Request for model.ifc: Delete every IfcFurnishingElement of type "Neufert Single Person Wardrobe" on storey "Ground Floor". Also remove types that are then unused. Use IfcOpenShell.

First a look at what the model holds.

```python
import ifcopenshell
import ifcopenshell.util.element

model = ifcopenshell.open("model.ifc")
print(model.schema)
storey = next(s for s in model.by_type("IfcBuildingStorey") if s.Name == "Ground Floor")
furniture = [e for e in ifcopenshell.util.element.get_decomposition(storey) if e.is_a("IfcFurnishingElement")]
seen = {}
for e in furniture:
    element_type = ifcopenshell.util.element.get_type(e)
    name = element_type.Name if element_type not in (None, e) else None
    seen[name] = seen.get(name, 0) + 1
for name, count in sorted(seen.items(), key=str):
    print(count, "x", name)
```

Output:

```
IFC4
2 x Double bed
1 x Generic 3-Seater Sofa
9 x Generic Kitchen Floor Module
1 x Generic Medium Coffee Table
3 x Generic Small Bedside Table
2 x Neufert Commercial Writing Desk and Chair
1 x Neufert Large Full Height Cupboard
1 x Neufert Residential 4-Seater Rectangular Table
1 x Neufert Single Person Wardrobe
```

```python
import ifcopenshell
import ifcopenshell.api.root
import ifcopenshell.util.element

model = ifcopenshell.open("model.ifc")

storey = next(s for s in model.by_type("IfcBuildingStorey") if s.Name == "Ground Floor")
furniture = [e for e in ifcopenshell.util.element.get_decomposition(storey) if e.is_a("IfcFurnishingElement")]
targets = [e for e in furniture if (t := ifcopenshell.util.element.get_type(e)) not in (None, e) and t.Name == "Neufert Single Person Wardrobe"]
types = {ifcopenshell.util.element.get_type(e) for e in targets} - {None, *targets}

for e in targets:
    ifcopenshell.api.root.remove_product(model, product=e)
print(len(targets), "removed")

unused = [t for t in types if not ifcopenshell.util.element.get_types(t)]
for t in unused:
    ifcopenshell.api.root.remove_product(model, product=t)
print(len(unused), "unused types removed")

model.write("model-out.ifc")
```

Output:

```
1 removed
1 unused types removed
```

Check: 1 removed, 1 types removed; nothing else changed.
